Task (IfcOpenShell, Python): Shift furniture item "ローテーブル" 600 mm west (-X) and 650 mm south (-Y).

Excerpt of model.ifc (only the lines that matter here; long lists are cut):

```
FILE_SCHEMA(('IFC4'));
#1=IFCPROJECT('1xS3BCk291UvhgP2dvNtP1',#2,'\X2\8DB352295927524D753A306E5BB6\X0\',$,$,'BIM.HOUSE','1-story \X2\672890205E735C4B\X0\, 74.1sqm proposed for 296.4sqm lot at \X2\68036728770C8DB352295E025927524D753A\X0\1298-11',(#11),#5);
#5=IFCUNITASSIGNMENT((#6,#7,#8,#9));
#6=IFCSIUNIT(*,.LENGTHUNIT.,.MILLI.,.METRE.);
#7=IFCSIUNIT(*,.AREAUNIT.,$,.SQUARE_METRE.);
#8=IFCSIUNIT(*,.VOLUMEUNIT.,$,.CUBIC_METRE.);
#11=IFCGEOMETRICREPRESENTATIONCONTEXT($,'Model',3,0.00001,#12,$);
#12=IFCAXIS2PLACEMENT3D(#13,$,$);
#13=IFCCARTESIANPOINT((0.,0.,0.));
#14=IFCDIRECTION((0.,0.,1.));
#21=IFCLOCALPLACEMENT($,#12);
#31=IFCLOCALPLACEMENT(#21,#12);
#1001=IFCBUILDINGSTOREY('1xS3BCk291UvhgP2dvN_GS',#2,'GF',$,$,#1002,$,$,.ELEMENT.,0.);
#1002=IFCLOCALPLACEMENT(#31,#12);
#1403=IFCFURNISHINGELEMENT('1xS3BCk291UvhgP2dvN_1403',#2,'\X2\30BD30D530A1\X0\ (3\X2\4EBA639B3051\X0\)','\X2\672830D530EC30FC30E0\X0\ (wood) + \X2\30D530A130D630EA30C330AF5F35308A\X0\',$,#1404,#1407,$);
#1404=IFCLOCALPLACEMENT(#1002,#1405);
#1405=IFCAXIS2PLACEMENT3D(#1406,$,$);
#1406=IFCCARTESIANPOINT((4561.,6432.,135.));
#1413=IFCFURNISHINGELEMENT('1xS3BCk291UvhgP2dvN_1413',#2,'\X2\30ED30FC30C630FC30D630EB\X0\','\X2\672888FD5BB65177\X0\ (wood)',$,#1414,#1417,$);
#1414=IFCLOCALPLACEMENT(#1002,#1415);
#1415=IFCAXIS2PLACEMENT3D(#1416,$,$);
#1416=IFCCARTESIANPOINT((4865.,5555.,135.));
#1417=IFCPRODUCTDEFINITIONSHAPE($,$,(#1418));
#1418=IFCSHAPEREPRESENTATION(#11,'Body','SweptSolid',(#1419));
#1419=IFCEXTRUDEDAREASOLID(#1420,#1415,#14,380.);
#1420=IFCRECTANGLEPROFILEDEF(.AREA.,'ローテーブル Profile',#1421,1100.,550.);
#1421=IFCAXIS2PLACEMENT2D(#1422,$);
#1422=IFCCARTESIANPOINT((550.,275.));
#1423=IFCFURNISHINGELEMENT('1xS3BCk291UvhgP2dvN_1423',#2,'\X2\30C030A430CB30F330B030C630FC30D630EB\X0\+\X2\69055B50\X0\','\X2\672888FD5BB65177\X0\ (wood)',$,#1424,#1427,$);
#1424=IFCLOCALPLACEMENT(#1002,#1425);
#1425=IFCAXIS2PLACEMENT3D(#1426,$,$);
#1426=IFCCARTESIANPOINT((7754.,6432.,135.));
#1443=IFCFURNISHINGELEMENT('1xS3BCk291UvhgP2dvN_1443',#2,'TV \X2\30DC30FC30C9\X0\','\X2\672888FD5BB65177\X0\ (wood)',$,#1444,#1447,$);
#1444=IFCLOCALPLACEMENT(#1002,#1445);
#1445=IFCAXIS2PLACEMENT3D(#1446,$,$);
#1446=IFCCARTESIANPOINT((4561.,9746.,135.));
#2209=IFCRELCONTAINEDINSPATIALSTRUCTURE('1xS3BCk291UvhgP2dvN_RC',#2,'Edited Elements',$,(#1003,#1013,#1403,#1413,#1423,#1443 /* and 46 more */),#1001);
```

```python
import ifcopenshell
import ifcopenshell.api.geometry
import ifcopenshell.util.placement
import ifcopenshell.util.unit

model = ifcopenshell.open("model.ifc")
unit_scale = ifcopenshell.util.unit.calculate_unit_scale(model)

item = model.by_id(1413)
matrix = ifcopenshell.util.placement.get_local_placement(item.ObjectPlacement)
matrix[0, 3] -= 0.6 / unit_scale
matrix[1, 3] -= 0.65 / unit_scale
ifcopenshell.api.geometry.edit_object_placement(model, product=item, matrix=matrix, is_si=False)

print(ifcopenshell.util.placement.get_local_placement(item.ObjectPlacement).round(3) + 0.0)

model.write("model-out.ifc")
```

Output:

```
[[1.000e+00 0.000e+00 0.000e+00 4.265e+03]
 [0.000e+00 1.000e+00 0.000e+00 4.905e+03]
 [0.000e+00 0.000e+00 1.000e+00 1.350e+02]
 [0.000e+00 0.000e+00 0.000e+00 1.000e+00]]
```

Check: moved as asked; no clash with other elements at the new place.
